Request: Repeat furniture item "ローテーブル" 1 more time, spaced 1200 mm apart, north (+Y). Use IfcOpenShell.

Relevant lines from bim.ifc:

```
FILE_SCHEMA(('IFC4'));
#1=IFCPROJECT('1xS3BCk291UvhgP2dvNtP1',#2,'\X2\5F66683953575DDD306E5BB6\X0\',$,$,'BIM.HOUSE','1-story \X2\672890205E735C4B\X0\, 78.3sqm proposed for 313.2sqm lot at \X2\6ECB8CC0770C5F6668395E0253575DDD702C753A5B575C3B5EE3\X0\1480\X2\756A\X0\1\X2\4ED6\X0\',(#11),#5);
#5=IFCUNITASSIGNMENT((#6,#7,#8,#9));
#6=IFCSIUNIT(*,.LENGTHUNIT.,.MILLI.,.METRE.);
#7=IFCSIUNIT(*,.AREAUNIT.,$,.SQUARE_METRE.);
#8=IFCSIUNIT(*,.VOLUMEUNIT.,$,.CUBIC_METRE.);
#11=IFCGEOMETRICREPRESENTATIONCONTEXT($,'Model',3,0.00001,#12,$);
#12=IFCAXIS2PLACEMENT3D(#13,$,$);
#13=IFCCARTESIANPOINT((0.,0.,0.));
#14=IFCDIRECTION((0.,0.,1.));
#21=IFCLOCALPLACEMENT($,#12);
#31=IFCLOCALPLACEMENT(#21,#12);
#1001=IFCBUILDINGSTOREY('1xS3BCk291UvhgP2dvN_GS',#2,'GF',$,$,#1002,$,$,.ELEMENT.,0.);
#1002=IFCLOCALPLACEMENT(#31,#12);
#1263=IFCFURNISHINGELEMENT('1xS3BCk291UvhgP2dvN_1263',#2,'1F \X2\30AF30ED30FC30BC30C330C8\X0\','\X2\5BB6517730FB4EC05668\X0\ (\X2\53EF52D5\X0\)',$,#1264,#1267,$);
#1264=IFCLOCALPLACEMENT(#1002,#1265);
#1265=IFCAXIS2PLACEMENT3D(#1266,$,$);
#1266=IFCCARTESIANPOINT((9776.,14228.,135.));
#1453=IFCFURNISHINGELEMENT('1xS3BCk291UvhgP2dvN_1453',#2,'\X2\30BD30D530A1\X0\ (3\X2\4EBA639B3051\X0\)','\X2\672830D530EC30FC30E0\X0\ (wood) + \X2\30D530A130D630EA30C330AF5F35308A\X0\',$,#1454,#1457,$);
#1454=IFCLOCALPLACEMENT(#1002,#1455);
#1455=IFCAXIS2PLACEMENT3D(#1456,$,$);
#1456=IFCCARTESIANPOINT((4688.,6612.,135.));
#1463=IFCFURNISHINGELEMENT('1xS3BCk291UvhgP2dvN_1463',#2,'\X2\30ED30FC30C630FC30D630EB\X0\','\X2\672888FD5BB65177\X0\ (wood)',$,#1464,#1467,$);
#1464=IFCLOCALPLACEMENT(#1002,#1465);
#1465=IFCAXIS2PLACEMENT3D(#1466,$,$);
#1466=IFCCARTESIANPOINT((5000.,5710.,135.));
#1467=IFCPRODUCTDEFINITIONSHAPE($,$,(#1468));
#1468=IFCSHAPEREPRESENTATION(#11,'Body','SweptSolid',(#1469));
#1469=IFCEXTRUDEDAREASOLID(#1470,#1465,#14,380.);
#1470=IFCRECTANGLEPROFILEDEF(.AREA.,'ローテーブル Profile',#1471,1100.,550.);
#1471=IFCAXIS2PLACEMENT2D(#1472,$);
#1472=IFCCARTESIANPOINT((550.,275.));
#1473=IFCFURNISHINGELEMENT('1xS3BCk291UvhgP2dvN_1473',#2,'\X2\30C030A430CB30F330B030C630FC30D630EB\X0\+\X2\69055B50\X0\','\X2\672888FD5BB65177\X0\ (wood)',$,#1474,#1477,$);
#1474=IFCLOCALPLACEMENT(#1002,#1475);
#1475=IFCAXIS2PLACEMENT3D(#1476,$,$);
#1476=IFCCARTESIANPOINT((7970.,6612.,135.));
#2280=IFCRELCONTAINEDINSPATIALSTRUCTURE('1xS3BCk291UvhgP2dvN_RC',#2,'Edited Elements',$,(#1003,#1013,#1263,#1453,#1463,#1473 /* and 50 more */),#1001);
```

```python
import numpy as np
import ifcopenshell
import ifcopenshell.api.geometry
import ifcopenshell.api.root
import ifcopenshell.util.element
import ifcopenshell.util.placement
import ifcopenshell.util.unit

model = ifcopenshell.open("bim.ifc")
unit_scale = ifcopenshell.util.unit.calculate_unit_scale(model)


def reuse_history(source, copy):
    """copy_class also copies each property set's owner history, people and application; keep the originals."""
    for rel in copy.IsDefinedBy:
        if rel.is_a("IfcRelDefinesByProperties") and (history := rel.RelatingPropertyDefinition.OwnerHistory):
            rel.RelatingPropertyDefinition.OwnerHistory = source.OwnerHistory
            ifcopenshell.util.element.remove_deep2(model, history)


source = model.by_id(1463)
base = ifcopenshell.util.placement.get_local_placement(source.ObjectPlacement)
step = np.array([0.0, 1.0, 0.0]) * 1.2 / unit_scale

for i in range(1, 2):
    copy = ifcopenshell.api.root.copy_class(model, product=source)
    copy.Representation = ifcopenshell.util.element.copy_deep(
        model, source.Representation, exclude=["IfcGeometricRepresentationContext", "IfcRepresentationMap"]
    )
    reuse_history(source, copy)
    matrix = base.copy()
    matrix[:3, 3] += i * step
    print("added at", matrix[:3, 3].round(3) + 0.0)
    ifcopenshell.api.geometry.edit_object_placement(model, product=copy, matrix=matrix, is_si=False)

model.write("bim_edited.ifc")
```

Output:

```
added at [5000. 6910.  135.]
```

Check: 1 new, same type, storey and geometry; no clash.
